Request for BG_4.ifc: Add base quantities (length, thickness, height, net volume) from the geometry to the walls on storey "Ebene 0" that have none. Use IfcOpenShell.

First a look at what the model holds.

```python
import ifcopenshell
import ifcopenshell.util.element
import ifcopenshell.util.unit

model = ifcopenshell.open("BG_4.ifc")
print(model.schema)
for unit_type in ("LENGTHUNIT", "AREAUNIT", "VOLUMEUNIT"):
    print(unit_type, ifcopenshell.util.unit.calculate_unit_scale(model, unit_type))
storey = next(s for s in model.by_type("IfcBuildingStorey") if s.Name == "Ebene 0")
walls = [e for e in ifcopenshell.util.element.get_decomposition(storey) if e.is_a("IfcWall")]
for e in sorted(walls, key=lambda e: e.id()):
    print(e.id(), e.is_a(), e.Name, list(ifcopenshell.util.element.get_psets(e, qtos_only=True)), sep=" | ")
```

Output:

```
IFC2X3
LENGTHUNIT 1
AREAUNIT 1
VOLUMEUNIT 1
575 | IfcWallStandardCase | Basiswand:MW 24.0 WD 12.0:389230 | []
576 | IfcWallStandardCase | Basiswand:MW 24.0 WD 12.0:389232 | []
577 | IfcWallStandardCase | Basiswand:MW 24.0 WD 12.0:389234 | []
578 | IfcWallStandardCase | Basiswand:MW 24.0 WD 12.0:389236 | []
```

```python
import ifcopenshell
import ifcopenshell.api.pset
import ifcopenshell.geom
import ifcopenshell.util.element
import ifcopenshell.util.shape
import ifcopenshell.util.unit

model = ifcopenshell.open("BG_4.ifc")
unit_scale = ifcopenshell.util.unit.calculate_unit_scale(model)
volume_scale = ifcopenshell.util.unit.calculate_unit_scale(model, "VOLUMEUNIT")
settings = ifcopenshell.geom.settings()

storey = next(s for s in model.by_type("IfcBuildingStorey") if s.Name == "Ebene 0")
walls = [e for e in ifcopenshell.util.element.get_decomposition(storey) if e.is_a("IfcWall")]

for e in sorted(walls, key=lambda e: e.id()):
    if ifcopenshell.util.element.get_psets(e, qtos_only=True, should_inherit=False):
        continue
    # Geometry comes back in metres, in the element's own axes.
    shape = ifcopenshell.geom.create_shape(settings, e)
    values = {
        "Length": ifcopenshell.util.shape.get_x(shape.geometry) / unit_scale,
        "Width": ifcopenshell.util.shape.get_y(shape.geometry) / unit_scale,
        "Height": ifcopenshell.util.shape.get_z(shape.geometry) / unit_scale,
        "NetVolume": ifcopenshell.util.shape.get_volume(shape.geometry) / volume_scale,
    }
    qto = ifcopenshell.api.pset.add_qto(model, product=e, name="BaseQuantities")
    ifcopenshell.api.pset.edit_qto(model, qto=qto, properties=values)
    print(e.id(), {k: round(v, 3) for k, v in values.items()})

model.write("BG_4_v2.ifc")
```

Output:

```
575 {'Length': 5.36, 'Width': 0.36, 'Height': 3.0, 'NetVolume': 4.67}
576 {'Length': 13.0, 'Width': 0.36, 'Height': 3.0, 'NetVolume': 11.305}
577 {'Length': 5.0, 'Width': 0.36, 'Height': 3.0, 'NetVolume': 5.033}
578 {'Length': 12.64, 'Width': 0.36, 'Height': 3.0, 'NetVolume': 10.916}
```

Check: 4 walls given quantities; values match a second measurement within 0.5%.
